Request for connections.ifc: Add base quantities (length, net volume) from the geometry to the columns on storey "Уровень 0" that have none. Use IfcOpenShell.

First a look at what the model holds.

```python
import ifcopenshell
import ifcopenshell.util.element
import ifcopenshell.util.unit

model = ifcopenshell.open("connections.ifc")
print(model.schema)
for unit_type in ("LENGTHUNIT", "AREAUNIT", "VOLUMEUNIT"):
    print(unit_type, ifcopenshell.util.unit.calculate_unit_scale(model, unit_type))
storey = next(s for s in model.by_type("IfcBuildingStorey") if s.Name == "Уровень 0")
columns = [e for e in ifcopenshell.util.element.get_decomposition(storey) if e.is_a("IfcColumn")]
for e in sorted(columns, key=lambda e: e.id()):
    print(e.id(), e.is_a(), e.Name, list(ifcopenshell.util.element.get_psets(e, qtos_only=True)), sep=" | ")
```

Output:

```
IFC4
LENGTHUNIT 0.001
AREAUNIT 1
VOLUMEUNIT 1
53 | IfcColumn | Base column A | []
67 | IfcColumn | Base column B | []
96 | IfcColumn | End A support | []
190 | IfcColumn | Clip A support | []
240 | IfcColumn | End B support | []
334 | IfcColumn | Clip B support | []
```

```python
import ifcopenshell
import ifcopenshell.api.pset
import ifcopenshell.geom
import ifcopenshell.util.element
import ifcopenshell.util.shape
import ifcopenshell.util.unit

model = ifcopenshell.open("connections.ifc")
unit_scale = ifcopenshell.util.unit.calculate_unit_scale(model)
volume_scale = ifcopenshell.util.unit.calculate_unit_scale(model, "VOLUMEUNIT")
settings = ifcopenshell.geom.settings()

storey = next(s for s in model.by_type("IfcBuildingStorey") if s.Name == "Уровень 0")
columns = [e for e in ifcopenshell.util.element.get_decomposition(storey) if e.is_a("IfcColumn")]

for e in sorted(columns, key=lambda e: e.id()):
    if ifcopenshell.util.element.get_psets(e, qtos_only=True, should_inherit=False):
        continue
    # Geometry comes back in metres, in the element's own axes.
    shape = ifcopenshell.geom.create_shape(settings, e)
    values = {
        "Length": ifcopenshell.util.shape.get_z(shape.geometry) / unit_scale,
        "NetVolume": ifcopenshell.util.shape.get_volume(shape.geometry) / volume_scale,
    }
    qto = ifcopenshell.api.pset.add_qto(model, product=e, name="Qto_ColumnBaseQuantities")
    ifcopenshell.api.pset.edit_qto(model, qto=qto, properties=values)
    print(e.id(), {k: round(v, 3) for k, v in values.items()})

model.write("connections-out.ifc")
```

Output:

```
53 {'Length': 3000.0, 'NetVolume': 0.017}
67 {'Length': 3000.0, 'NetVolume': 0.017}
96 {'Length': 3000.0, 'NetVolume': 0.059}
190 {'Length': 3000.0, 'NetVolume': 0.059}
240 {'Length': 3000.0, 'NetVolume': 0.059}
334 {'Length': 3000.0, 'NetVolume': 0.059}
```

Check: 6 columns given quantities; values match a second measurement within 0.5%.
